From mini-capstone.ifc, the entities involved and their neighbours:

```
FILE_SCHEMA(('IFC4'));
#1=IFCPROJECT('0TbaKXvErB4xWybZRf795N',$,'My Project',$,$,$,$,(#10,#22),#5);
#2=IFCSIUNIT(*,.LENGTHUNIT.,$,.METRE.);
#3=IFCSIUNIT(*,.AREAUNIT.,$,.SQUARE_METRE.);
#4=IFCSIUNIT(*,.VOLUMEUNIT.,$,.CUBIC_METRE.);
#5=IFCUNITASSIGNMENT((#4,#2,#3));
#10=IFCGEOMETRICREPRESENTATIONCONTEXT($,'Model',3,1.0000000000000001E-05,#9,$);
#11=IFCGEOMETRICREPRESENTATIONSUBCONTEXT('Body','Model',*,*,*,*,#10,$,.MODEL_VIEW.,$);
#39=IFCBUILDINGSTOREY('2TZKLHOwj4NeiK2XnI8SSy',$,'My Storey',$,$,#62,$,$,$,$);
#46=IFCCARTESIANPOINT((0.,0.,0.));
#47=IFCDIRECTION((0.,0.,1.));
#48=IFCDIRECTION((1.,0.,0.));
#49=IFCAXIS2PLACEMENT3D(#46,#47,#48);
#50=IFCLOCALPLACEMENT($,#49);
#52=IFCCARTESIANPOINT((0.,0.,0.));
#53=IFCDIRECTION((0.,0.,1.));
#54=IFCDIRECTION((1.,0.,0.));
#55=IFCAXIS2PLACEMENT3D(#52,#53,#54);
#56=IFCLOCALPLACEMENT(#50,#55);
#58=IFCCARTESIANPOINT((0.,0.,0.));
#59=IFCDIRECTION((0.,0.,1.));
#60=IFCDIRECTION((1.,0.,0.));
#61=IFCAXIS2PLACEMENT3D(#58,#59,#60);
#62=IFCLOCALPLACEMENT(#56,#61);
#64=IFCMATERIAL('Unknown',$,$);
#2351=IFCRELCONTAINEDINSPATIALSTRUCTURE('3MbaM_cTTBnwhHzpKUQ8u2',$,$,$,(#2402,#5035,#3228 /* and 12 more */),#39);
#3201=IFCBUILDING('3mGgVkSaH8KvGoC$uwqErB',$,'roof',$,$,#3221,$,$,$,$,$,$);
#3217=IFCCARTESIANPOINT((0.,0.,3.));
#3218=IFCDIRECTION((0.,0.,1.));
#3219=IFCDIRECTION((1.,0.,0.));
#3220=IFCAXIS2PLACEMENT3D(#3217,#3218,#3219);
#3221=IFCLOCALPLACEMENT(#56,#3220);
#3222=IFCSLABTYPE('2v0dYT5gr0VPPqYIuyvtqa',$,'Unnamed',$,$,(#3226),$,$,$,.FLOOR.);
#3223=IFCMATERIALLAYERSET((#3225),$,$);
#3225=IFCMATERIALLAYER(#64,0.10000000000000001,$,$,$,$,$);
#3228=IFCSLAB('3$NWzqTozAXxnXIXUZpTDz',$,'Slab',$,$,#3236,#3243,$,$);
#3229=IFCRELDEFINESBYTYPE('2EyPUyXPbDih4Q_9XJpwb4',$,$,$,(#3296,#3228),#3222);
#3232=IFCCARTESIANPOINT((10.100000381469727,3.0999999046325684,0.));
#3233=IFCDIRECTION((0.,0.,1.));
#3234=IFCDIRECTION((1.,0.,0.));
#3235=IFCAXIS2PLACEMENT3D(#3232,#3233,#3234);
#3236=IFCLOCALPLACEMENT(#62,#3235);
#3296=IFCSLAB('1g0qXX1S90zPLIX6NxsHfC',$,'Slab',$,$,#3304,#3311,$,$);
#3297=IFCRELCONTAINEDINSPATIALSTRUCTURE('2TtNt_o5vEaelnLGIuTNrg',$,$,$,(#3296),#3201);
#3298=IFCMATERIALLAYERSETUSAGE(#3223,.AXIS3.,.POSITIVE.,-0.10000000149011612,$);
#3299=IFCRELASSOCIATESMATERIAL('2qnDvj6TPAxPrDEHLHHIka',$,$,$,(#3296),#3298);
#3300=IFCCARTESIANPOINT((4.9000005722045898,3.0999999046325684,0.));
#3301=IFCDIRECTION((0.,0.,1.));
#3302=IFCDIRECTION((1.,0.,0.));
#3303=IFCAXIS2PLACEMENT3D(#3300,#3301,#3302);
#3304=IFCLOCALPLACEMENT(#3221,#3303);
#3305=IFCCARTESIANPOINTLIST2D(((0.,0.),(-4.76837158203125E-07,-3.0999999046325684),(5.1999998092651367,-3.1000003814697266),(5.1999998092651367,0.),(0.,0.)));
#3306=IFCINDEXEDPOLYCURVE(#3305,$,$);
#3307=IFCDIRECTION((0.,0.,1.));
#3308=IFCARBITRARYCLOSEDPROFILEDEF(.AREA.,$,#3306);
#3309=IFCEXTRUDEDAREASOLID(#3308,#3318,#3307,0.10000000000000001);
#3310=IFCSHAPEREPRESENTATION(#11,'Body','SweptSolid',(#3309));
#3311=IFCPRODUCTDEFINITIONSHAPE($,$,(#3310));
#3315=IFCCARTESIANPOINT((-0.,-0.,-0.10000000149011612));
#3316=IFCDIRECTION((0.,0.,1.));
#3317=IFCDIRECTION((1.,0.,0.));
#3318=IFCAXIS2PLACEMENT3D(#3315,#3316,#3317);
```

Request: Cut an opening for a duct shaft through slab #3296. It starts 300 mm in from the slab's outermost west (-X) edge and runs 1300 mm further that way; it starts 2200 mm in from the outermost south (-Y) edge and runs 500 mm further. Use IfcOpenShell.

```python
import numpy as np
import ifcopenshell
import ifcopenshell.api.feature
import ifcopenshell.api.geometry
import ifcopenshell.api.root
import ifcopenshell.geom
import ifcopenshell.util.placement
import ifcopenshell.util.representation
import ifcopenshell.util.shape
import ifcopenshell.util.unit

model = ifcopenshell.open("mini-capstone.ifc")
unit_scale = ifcopenshell.util.unit.calculate_unit_scale(model)
settings = ifcopenshell.geom.settings()


def volume(element):
    """Net volume in cubic metres, openings subtracted."""
    shape = ifcopenshell.geom.create_shape(settings, element)
    return ifcopenshell.util.shape.get_volume(shape.geometry)


slab = model.by_guid("1g0qXX1S90zPLIX6NxsHfC")
before = volume(slab)

# Extent in the slab's own axes, in metres. The edges named are its -X and -Y sides.
slab_shape = ifcopenshell.geom.create_shape(settings, slab)
vertices = ifcopenshell.util.shape.get_vertices(slab_shape.geometry)
x_min, y_min, bottom = vertices.min(axis=0)
top = vertices[:, 2].max()

opening = ifcopenshell.api.root.create_entity(model, ifc_class="IfcOpeningElement", name="Duct shaft opening", predefined_type="OPENING")
context = ifcopenshell.util.representation.get_context(model, "Model", "Body", "MODEL_VIEW")
width, depth = 1.3, 0.5
outline = [(0.0, 0.0), (width, 0.0), (width, depth), (0.0, depth), (0.0, 0.0)]
# Overshoot both faces by 50 mm so the cut is clean.
shape = ifcopenshell.api.geometry.add_slab_representation(
    model, context=context, depth=top - bottom + 0.1, polyline=outline
)
ifcopenshell.api.geometry.assign_representation(model, product=opening, representation=shape)

matrix = ifcopenshell.util.placement.get_local_placement(slab.ObjectPlacement)
matrix[:, 3] = matrix @ np.append(np.array([x_min + 0.3, y_min + 2.2, bottom - 0.05]) / unit_scale, 1.0)
ifcopenshell.api.geometry.edit_object_placement(model, product=opening, matrix=matrix, is_si=False)
ifcopenshell.api.feature.add_feature(model, feature=opening, element=slab)

after = volume(slab)

print(f"slab volume {before:.3f} -> {after:.3f} m3")

model.write("mini-capstone_rev.ifc")
```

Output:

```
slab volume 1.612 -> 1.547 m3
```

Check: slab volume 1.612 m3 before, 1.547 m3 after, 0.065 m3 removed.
